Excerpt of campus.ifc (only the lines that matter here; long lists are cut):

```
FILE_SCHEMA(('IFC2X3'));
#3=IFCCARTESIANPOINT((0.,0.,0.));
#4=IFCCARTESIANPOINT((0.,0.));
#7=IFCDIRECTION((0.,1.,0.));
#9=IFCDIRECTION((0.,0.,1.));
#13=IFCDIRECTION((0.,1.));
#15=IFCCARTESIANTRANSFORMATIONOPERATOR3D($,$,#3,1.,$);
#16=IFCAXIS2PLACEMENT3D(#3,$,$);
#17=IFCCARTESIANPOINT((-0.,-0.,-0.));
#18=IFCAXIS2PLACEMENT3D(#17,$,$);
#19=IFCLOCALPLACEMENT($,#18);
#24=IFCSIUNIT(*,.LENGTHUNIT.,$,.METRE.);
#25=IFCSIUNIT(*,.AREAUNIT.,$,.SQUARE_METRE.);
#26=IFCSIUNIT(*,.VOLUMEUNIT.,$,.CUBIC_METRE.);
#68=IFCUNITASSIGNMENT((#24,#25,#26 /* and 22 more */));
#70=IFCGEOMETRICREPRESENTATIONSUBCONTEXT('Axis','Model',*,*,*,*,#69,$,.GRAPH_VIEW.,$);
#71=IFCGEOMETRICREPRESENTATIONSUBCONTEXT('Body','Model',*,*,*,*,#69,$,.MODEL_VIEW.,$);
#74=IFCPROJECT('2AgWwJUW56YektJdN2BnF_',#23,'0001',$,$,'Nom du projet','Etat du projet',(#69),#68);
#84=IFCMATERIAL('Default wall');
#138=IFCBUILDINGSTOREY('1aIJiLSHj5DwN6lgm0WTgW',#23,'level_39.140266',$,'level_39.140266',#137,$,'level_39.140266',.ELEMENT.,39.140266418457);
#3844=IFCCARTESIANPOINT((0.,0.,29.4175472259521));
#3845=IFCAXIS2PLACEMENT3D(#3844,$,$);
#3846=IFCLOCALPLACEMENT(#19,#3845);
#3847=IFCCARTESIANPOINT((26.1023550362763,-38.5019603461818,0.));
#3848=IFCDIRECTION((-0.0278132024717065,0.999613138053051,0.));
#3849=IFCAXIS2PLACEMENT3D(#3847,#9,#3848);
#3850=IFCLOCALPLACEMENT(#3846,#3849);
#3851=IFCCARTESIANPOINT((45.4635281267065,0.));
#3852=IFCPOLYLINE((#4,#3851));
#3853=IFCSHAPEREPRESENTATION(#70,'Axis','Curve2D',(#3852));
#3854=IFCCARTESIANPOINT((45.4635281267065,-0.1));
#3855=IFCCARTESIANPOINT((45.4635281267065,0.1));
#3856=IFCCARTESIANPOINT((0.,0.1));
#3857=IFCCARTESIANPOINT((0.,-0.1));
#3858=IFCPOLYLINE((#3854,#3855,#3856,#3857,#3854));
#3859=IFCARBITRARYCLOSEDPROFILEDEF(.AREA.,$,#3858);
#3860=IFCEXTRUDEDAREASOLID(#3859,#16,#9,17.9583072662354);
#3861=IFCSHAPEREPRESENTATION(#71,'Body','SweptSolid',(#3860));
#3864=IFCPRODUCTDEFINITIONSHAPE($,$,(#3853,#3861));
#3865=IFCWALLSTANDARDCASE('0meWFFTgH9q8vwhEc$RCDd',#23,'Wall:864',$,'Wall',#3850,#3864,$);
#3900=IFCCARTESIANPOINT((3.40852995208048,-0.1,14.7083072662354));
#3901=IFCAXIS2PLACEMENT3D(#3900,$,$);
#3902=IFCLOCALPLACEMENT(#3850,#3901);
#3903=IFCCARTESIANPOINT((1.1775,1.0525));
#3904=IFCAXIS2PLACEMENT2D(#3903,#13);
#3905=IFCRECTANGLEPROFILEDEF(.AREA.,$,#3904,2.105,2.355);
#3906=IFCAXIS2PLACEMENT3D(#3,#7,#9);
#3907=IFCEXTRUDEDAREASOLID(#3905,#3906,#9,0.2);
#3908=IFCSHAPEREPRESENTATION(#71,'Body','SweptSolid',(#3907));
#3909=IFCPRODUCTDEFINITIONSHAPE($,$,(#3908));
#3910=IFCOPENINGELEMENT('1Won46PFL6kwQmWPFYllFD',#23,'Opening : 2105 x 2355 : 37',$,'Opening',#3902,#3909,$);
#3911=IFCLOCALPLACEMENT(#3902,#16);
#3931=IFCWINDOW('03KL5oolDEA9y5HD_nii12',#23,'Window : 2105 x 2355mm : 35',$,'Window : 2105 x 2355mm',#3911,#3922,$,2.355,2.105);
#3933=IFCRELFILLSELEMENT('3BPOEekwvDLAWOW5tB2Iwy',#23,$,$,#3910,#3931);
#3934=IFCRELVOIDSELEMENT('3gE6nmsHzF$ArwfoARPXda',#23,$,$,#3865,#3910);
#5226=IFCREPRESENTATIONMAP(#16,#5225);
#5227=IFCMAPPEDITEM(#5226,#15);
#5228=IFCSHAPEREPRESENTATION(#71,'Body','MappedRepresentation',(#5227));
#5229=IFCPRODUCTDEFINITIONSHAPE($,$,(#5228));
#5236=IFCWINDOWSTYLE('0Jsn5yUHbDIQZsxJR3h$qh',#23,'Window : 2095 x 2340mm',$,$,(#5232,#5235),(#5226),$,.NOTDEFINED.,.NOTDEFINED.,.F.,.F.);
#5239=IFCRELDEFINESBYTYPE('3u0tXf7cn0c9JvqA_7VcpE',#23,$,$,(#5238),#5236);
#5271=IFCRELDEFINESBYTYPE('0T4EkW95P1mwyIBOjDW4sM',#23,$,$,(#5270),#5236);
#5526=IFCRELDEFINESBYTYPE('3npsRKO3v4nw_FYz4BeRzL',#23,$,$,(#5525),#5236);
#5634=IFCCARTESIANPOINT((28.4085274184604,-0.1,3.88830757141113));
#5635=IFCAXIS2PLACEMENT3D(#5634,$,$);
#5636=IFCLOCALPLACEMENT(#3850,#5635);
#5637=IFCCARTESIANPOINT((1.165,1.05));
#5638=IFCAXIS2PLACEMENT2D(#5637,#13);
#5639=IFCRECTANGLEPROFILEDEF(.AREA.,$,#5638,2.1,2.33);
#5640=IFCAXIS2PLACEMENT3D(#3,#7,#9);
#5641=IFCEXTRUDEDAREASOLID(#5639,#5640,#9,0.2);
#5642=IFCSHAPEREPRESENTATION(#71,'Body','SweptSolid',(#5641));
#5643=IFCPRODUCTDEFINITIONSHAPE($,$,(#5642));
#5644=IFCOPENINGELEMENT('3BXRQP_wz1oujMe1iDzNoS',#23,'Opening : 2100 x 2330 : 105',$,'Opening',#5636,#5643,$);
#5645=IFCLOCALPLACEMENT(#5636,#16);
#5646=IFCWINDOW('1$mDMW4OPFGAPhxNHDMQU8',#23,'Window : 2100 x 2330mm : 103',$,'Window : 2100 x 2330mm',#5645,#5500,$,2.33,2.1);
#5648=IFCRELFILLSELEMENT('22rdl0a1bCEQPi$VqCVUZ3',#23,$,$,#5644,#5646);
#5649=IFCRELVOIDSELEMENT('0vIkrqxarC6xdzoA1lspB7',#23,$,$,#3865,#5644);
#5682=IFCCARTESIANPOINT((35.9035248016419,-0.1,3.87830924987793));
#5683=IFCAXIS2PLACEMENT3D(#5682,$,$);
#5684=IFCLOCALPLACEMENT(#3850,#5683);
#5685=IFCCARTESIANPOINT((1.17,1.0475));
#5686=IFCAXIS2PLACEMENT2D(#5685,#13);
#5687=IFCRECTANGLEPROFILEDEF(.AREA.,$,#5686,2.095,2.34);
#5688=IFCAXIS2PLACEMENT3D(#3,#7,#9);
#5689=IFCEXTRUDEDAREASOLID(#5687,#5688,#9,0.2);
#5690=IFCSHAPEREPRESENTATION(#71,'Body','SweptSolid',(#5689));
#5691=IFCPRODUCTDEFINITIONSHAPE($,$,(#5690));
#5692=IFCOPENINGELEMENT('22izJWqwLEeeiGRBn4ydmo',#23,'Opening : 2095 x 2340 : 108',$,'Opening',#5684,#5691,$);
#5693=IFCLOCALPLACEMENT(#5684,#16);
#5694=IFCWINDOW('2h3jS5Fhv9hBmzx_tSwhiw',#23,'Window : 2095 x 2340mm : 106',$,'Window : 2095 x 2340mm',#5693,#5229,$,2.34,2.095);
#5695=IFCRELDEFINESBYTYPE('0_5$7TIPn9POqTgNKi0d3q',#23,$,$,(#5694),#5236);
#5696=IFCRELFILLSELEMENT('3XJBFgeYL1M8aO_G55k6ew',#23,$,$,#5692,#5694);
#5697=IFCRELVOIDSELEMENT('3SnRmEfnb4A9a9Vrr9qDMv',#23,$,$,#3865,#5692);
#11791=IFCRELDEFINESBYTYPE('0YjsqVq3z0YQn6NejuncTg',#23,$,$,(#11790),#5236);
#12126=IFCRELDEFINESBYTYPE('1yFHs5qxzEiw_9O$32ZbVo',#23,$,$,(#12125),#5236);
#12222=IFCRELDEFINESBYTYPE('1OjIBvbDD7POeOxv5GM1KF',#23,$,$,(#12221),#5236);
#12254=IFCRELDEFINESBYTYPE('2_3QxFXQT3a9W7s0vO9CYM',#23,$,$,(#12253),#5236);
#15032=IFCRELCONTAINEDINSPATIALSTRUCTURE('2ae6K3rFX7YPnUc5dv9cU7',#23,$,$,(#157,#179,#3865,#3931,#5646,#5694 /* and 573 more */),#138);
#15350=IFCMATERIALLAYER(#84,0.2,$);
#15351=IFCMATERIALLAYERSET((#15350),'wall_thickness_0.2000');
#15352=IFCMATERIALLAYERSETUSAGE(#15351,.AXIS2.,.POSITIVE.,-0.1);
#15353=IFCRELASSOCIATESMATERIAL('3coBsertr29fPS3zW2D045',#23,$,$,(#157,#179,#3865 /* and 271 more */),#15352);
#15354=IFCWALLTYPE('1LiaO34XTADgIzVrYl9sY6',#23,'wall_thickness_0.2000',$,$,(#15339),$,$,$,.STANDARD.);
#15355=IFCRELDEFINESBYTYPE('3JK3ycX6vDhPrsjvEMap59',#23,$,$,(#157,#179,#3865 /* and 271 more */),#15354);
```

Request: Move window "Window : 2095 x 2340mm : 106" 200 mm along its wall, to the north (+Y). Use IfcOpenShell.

```python
import ifcopenshell
import ifcopenshell.api.geometry
import ifcopenshell.util.placement
import ifcopenshell.util.unit

model = ifcopenshell.open("campus.ifc")
unit_scale = ifcopenshell.util.unit.calculate_unit_scale(model)

window = model.by_guid("2h3jS5Fhv9hBmzx_tSwhiw")
opening = window.FillsVoids[0].RelatingOpeningElement
wall = opening.VoidsElements[0].RelatingBuildingElement

wall_matrix = ifcopenshell.util.placement.get_local_placement(wall.ObjectPlacement)
shift = wall_matrix[:3, 0] * 0.2 / unit_scale
before = ifcopenshell.util.placement.get_local_placement(window.ObjectPlacement)[:3, 3].copy()

# The window is placed relative to its opening, so it follows when the opening moves.
matrix = ifcopenshell.util.placement.get_local_placement(opening.ObjectPlacement)
matrix[:3, 3] += shift
ifcopenshell.api.geometry.edit_object_placement(
    model, product=opening, matrix=matrix, is_si=False, should_transform_children=True
)

after = ifcopenshell.util.placement.get_local_placement(window.ObjectPlacement)[:3, 3]
print("window moved by", (after - before).round(3) + 0.0)

model.write("campus-out.ifc")
```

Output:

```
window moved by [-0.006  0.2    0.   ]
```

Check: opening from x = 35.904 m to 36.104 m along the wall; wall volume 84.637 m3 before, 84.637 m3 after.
